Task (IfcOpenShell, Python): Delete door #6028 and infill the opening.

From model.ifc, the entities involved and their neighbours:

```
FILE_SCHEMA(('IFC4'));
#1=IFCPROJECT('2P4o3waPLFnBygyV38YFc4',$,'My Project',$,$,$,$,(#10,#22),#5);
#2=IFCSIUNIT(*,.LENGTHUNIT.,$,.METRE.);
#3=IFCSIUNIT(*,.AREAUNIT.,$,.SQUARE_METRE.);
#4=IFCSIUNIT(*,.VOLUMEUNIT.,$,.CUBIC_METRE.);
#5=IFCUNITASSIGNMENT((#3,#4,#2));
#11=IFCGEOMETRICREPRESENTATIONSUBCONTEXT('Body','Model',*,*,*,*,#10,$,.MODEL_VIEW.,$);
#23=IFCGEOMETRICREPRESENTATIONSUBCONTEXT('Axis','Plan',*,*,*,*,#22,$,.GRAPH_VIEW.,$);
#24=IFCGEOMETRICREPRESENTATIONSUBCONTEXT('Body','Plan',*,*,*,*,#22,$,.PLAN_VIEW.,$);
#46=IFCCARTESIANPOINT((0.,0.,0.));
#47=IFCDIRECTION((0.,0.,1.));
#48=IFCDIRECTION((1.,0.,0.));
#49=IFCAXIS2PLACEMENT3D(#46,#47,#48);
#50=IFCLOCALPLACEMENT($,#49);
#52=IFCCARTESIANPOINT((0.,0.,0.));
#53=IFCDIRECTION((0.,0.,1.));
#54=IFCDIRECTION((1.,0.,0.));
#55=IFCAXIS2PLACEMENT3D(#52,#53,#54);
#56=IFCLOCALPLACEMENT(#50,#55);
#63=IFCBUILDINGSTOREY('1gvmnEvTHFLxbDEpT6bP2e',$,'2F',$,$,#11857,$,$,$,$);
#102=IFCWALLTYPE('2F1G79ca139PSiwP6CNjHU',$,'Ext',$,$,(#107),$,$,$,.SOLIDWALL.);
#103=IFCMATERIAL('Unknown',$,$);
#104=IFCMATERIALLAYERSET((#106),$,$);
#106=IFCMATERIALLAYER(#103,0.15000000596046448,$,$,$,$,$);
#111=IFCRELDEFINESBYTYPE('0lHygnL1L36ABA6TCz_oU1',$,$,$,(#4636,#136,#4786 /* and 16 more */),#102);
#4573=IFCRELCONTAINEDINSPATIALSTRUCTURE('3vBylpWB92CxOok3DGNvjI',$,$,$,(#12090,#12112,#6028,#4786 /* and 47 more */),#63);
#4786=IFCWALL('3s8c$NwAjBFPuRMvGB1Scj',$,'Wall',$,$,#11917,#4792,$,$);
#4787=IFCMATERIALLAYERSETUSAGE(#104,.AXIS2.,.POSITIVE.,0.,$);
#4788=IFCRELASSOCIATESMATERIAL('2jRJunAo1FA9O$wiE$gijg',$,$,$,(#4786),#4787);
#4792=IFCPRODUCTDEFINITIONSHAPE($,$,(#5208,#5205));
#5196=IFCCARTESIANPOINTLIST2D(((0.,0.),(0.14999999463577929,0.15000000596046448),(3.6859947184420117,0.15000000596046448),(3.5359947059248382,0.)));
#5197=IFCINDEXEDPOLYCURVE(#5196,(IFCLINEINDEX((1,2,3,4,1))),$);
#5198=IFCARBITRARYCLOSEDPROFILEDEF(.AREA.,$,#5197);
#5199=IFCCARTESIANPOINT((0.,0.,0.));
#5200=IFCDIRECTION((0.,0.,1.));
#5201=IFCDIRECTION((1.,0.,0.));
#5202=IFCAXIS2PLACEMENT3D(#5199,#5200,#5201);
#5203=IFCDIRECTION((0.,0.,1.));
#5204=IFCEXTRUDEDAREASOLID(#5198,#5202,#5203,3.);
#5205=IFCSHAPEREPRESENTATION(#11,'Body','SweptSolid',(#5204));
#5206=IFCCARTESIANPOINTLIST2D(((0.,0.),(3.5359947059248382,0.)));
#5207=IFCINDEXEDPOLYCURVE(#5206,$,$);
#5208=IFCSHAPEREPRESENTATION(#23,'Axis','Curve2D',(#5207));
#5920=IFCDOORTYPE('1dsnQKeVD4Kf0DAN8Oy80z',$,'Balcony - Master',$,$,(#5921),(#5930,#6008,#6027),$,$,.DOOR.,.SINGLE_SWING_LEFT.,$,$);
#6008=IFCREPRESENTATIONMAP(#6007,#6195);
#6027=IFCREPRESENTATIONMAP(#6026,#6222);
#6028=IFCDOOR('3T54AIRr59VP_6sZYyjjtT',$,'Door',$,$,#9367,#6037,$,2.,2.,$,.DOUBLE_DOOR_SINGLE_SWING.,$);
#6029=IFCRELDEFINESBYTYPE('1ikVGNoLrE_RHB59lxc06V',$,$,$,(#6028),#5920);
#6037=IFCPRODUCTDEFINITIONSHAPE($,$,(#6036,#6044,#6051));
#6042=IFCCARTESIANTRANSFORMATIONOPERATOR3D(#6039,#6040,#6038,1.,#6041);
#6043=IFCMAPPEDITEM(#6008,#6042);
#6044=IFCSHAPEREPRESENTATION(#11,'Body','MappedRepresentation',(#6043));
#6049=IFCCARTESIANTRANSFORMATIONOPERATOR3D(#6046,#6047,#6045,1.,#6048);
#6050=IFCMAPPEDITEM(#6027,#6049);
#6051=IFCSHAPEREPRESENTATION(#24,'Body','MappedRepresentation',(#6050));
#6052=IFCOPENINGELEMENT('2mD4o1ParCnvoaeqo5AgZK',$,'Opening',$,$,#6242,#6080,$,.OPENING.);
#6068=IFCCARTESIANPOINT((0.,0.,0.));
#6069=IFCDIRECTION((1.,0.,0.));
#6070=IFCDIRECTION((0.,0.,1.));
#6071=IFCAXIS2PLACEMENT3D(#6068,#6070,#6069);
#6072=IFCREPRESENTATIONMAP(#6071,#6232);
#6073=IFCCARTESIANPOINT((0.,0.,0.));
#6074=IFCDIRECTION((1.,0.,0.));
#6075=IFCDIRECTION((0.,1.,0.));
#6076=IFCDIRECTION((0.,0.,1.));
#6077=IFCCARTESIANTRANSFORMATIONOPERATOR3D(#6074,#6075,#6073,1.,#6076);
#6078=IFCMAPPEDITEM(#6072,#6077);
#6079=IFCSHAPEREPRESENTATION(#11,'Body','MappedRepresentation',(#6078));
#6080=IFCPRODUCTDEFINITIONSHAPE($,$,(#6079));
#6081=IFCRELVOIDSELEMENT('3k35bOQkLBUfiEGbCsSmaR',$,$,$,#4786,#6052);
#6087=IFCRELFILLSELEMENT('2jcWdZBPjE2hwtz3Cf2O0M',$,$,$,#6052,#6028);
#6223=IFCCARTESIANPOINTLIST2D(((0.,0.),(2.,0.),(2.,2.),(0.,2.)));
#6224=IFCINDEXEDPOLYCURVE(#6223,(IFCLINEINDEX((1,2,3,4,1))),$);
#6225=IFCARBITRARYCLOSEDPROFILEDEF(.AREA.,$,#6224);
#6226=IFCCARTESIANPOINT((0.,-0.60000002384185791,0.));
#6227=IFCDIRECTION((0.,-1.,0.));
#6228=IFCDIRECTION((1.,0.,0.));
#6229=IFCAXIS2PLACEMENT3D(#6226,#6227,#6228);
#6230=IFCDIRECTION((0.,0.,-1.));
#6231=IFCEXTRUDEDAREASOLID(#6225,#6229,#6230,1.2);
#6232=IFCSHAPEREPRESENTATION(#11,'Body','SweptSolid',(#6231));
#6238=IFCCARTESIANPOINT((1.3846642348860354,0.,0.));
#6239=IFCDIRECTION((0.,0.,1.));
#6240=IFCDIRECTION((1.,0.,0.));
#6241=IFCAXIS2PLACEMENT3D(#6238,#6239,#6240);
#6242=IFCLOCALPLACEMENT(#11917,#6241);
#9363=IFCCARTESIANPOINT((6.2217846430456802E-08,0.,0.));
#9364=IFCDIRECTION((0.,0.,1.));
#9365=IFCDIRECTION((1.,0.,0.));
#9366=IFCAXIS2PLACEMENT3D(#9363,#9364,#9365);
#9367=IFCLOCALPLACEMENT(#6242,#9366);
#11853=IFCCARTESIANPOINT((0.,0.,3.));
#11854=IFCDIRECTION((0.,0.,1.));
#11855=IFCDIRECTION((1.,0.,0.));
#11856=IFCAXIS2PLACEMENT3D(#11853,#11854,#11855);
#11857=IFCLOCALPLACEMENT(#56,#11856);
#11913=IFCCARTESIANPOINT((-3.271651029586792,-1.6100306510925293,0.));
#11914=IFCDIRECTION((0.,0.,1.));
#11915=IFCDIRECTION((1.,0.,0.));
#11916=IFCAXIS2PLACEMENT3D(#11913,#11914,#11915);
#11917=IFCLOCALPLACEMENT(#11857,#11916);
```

```python
import ifcopenshell
import ifcopenshell.api.feature
import ifcopenshell.api.root
import ifcopenshell.geom
import ifcopenshell.util.shape

model = ifcopenshell.open("model.ifc")
settings = ifcopenshell.geom.settings()


def volume(element):
    """Net volume in cubic metres, openings subtracted."""
    shape = ifcopenshell.geom.create_shape(settings, element)
    return ifcopenshell.util.shape.get_volume(shape.geometry)


door = model.by_guid("3T54AIRr59VP_6sZYyjjtT")
opening = door.FillsVoids[0].RelatingOpeningElement
wall = opening.VoidsElements[0].RelatingBuildingElement
before = volume(wall)

ifcopenshell.api.root.remove_product(model, product=door)
ifcopenshell.api.feature.remove_feature(model, feature=opening)

after = volume(wall)

print(f"wall volume {before:.3f} -> {after:.3f} m3")

model.write("model_rev.ifc")
```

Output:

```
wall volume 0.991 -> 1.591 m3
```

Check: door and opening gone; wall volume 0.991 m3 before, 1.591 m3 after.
